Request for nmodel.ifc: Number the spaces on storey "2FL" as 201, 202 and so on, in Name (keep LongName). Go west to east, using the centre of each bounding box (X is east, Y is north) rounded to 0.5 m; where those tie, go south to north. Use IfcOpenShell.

First a look at what the model holds.

```python
import ifcopenshell
import ifcopenshell.util.element
import ifcopenshell.util.placement

model = ifcopenshell.open("nmodel.ifc")
print(model.schema)
storey = next(s for s in model.by_type("IfcBuildingStorey") if s.Name == "2FL")
spaces = [e for e in ifcopenshell.util.element.get_decomposition(storey) if e.is_a("IfcSpace")]
for e in sorted(spaces, key=lambda e: e.id()):
    origin = ifcopenshell.util.placement.get_local_placement(e.ObjectPlacement)[:3, 3]
    print(e.id(), e.Name, e.LongName, origin.round(2) + 0.0, sep=" | ")
```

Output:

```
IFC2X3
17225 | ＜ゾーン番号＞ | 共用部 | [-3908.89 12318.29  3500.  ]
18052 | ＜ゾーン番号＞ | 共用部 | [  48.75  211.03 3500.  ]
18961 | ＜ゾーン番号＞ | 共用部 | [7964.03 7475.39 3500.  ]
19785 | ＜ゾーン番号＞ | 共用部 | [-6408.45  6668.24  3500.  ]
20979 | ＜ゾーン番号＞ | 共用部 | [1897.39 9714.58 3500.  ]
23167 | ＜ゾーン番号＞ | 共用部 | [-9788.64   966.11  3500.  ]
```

```python
import ifcopenshell
import ifcopenshell.geom
import ifcopenshell.util.element
import ifcopenshell.util.shape

model = ifcopenshell.open("nmodel.ifc")
settings = ifcopenshell.geom.settings()
settings.set("use-world-coords", True)


def centre(element):
    shape = ifcopenshell.geom.create_shape(settings, element)
    return ifcopenshell.util.shape.get_bbox_centroid(shape.geometry)


storey = next(s for s in model.by_type("IfcBuildingStorey") if s.Name == "2FL")
spaces = [e for e in ifcopenshell.util.element.get_decomposition(storey) if e.is_a("IfcSpace")]

# Insertion points can sit at a corner or the storey origin, so sort by the geometry (in metres).
centres = {e: centre(e) for e in spaces}
spaces.sort(key=lambda e: (round(centres[e][0] / 0.5), centres[e][1]))

for i, e in enumerate(spaces, start=1):
    number = f"2{i:02d}"
    e.Name = number
    print(e.id(), number)

model.write("nmodel_edited.ifc")
```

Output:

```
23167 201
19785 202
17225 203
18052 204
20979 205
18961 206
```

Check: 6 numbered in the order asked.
